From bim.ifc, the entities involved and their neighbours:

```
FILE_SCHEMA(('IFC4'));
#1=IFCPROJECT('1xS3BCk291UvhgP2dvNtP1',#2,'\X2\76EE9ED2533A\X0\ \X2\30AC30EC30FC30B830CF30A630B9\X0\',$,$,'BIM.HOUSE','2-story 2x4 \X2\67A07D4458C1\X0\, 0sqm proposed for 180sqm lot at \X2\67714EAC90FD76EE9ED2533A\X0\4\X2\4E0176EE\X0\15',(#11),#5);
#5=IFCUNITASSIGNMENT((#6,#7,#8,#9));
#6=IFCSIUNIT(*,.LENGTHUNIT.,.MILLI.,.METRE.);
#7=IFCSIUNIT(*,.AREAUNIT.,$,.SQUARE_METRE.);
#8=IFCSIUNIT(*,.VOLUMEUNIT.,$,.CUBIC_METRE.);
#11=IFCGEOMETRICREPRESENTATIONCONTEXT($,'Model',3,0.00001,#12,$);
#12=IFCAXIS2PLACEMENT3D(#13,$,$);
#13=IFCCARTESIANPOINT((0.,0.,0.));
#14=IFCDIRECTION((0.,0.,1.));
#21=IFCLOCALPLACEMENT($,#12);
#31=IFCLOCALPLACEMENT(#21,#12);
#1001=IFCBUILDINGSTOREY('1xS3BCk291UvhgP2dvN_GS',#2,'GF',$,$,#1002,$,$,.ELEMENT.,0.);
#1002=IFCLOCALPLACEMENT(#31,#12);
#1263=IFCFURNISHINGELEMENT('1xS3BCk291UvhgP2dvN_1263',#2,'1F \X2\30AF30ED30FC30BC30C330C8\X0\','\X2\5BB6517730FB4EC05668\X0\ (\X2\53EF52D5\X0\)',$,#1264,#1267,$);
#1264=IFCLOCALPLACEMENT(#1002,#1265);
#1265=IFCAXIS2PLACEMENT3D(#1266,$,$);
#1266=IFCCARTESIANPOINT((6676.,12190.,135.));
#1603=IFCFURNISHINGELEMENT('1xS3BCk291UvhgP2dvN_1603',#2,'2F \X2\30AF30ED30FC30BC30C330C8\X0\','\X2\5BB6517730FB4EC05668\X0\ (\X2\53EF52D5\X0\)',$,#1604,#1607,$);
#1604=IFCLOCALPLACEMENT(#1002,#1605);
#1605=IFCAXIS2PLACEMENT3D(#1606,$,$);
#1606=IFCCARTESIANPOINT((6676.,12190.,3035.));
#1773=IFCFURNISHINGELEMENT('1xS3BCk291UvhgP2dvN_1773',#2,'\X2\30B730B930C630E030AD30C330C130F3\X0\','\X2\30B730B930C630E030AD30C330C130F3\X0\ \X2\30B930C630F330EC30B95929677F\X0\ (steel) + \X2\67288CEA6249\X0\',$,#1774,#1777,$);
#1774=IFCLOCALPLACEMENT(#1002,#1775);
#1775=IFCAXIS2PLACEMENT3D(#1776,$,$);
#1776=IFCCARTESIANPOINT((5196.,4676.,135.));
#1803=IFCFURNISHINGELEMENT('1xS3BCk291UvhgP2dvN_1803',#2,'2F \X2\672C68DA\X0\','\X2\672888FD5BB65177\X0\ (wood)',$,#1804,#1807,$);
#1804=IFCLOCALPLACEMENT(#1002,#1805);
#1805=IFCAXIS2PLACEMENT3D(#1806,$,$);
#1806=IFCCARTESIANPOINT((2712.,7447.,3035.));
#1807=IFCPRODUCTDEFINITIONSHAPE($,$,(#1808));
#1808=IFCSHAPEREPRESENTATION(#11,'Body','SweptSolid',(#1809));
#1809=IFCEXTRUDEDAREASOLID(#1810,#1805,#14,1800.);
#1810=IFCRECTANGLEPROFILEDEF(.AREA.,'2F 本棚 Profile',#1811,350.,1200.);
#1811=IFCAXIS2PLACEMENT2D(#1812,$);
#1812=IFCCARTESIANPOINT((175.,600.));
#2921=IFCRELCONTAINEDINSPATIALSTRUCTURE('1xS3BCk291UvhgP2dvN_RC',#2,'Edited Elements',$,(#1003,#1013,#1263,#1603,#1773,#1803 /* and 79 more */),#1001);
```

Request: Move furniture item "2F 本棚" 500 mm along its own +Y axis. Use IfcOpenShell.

```python
import ifcopenshell
import ifcopenshell.api.geometry
import ifcopenshell.util.placement

model = ifcopenshell.open("bim.ifc")

item = model.by_id(1803)
matrix = ifcopenshell.util.placement.get_local_placement(item.ObjectPlacement)
matrix[:3, 3] += matrix[:3, 1] * 500.0
ifcopenshell.api.geometry.edit_object_placement(model, product=item, matrix=matrix, is_si=False)

print(ifcopenshell.util.placement.get_local_placement(item.ObjectPlacement).round(3) + 0.0)

model.write("bim_updated.ifc")
```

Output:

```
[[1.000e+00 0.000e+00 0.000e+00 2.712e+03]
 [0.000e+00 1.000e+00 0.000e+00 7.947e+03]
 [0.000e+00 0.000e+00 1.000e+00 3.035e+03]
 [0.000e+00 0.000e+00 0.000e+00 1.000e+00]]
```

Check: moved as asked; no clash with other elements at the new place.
